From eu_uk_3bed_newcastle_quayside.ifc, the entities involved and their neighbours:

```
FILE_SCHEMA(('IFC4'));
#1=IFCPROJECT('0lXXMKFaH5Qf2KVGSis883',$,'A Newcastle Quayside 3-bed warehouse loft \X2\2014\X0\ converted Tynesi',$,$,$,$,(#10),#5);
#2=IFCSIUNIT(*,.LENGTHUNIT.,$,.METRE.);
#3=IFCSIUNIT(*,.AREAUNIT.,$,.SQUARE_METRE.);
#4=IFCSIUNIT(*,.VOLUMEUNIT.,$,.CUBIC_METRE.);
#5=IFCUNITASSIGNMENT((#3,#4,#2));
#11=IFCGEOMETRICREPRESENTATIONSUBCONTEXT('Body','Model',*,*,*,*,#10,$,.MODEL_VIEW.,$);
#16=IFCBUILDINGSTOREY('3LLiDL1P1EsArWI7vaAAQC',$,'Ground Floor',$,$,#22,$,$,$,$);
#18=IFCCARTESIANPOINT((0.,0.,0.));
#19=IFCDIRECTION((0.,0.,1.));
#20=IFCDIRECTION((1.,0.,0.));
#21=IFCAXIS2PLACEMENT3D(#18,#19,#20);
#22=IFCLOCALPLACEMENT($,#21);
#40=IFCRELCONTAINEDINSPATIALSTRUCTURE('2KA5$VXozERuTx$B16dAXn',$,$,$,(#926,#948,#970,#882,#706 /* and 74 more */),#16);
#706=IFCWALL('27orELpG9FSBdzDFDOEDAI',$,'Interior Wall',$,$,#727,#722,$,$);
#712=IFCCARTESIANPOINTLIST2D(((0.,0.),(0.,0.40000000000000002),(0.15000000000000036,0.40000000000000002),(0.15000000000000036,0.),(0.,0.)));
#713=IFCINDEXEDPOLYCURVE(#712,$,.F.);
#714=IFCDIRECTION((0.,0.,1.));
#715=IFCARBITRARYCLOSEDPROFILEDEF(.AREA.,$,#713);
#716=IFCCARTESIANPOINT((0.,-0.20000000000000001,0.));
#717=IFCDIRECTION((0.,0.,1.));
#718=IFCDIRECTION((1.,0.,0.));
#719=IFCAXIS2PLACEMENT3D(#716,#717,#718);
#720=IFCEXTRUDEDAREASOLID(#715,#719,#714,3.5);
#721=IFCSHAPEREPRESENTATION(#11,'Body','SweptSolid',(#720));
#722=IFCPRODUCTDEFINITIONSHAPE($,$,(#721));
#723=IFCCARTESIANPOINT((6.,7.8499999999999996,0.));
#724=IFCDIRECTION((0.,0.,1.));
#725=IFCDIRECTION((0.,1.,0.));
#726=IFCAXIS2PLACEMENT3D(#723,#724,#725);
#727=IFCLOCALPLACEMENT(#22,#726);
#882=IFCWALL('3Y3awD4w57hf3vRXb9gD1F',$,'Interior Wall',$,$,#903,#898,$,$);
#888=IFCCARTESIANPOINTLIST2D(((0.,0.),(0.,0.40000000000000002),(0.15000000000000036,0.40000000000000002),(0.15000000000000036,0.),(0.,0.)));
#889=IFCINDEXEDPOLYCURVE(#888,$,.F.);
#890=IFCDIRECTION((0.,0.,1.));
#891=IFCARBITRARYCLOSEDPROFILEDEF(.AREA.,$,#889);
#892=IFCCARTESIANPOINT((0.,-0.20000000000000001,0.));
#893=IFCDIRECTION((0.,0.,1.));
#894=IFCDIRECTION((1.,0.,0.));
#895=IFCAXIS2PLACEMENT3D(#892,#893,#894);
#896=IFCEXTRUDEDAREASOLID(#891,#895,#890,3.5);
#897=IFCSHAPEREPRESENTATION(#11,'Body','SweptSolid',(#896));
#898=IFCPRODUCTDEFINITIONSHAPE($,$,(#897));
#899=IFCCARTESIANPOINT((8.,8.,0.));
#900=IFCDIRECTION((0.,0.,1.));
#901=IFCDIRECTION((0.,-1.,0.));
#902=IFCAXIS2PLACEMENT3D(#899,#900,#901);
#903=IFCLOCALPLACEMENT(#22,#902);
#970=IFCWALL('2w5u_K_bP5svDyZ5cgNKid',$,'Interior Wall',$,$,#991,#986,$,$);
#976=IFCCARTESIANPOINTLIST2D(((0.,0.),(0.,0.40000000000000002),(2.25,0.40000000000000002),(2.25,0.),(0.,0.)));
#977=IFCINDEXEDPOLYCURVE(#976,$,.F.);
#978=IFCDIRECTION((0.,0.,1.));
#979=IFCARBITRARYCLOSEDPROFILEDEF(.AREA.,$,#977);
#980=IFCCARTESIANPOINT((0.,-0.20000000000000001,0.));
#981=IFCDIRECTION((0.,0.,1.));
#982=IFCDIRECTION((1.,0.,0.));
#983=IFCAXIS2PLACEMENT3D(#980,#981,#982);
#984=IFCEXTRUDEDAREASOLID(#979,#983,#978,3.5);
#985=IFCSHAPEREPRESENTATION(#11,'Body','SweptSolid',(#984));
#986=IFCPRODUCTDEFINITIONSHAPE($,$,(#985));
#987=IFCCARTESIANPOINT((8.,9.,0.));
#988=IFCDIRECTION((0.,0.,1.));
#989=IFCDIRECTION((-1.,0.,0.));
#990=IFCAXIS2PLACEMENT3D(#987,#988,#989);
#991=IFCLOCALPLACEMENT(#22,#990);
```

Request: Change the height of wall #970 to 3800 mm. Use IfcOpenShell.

```python
import ifcopenshell
import ifcopenshell.geom
import ifcopenshell.util.representation
import ifcopenshell.util.shape
import ifcopenshell.util.unit

model = ifcopenshell.open("eu_uk_3bed_newcastle_quayside.ifc")
unit_scale = ifcopenshell.util.unit.calculate_unit_scale(model)
settings = ifcopenshell.geom.settings()


def volume(element):
    """Net volume in cubic metres, openings subtracted."""
    shape = ifcopenshell.geom.create_shape(settings, element)
    return ifcopenshell.util.shape.get_volume(shape.geometry)


wall = model.by_guid("2w5u_K_bP5svDyZ5cgNKid")
before = volume(wall)

body = ifcopenshell.util.representation.get_representation(wall, "Model", "Body")
solid = body.Items[0]
old_height = solid.Depth
solid.Depth = 3.8 / unit_scale
after = volume(wall)

print(f"height {old_height:g} -> {solid.Depth:g}, volume {before:.3f} -> {after:.3f} m3")

model.write("eu_uk_3bed_newcastle_quayside_rev.ifc")
```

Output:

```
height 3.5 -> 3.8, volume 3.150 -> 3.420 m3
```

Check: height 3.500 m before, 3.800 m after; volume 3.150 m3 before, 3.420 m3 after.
